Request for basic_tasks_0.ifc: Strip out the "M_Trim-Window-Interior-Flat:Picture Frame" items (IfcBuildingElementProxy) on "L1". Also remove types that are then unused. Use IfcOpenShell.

First a look at what the model holds.

```python
import ifcopenshell
import ifcopenshell.util.element

model = ifcopenshell.open("basic_tasks_0.ifc")
print(model.schema)
storey = next(s for s in model.by_type("IfcBuildingStorey") if s.Name == "L1")
proxies = [e for e in ifcopenshell.util.element.get_decomposition(storey) if e.is_a("IfcBuildingElementProxy")]
seen = {}
for e in proxies:
    element_type = ifcopenshell.util.element.get_type(e)
    name = element_type.Name if element_type not in (None, e) else None
    seen[name] = seen.get(name, 0) + 1
for name, count in sorted(seen.items(), key=str):
    print(count, "x", name)
```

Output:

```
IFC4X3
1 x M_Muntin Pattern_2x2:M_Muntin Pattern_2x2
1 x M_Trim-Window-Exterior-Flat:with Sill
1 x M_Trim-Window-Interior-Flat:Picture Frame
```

```python
import ifcopenshell
import ifcopenshell.api.root
import ifcopenshell.util.element

model = ifcopenshell.open("basic_tasks_0.ifc")

storey = next(s for s in model.by_type("IfcBuildingStorey") if s.Name == "L1")
proxies = [e for e in ifcopenshell.util.element.get_decomposition(storey) if e.is_a("IfcBuildingElementProxy")]
targets = [e for e in proxies if (t := ifcopenshell.util.element.get_type(e)) not in (None, e) and t.Name == "M_Trim-Window-Interior-Flat:Picture Frame"]
types = {ifcopenshell.util.element.get_type(e) for e in targets} - {None, *targets}

for e in targets:
    ifcopenshell.api.root.remove_product(model, product=e)
print(len(targets), "removed")

unused = [t for t in types if not ifcopenshell.util.element.get_types(t)]
for t in unused:
    ifcopenshell.api.root.remove_product(model, product=t)
print(len(unused), "unused types removed")

model.write("basic_tasks_0_edited.ifc")
```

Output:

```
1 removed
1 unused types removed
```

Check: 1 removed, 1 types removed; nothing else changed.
